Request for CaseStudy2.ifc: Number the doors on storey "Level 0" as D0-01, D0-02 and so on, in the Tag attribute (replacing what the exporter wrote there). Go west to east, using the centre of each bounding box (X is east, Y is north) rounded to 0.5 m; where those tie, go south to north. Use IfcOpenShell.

First a look at what the model holds.

```python
import ifcopenshell
import ifcopenshell.util.element
import ifcopenshell.util.placement

model = ifcopenshell.open("CaseStudy2.ifc")
print(model.schema)
storey = next(s for s in model.by_type("IfcBuildingStorey") if s.Name == "Level 0")
doors = [e for e in ifcopenshell.util.element.get_decomposition(storey) if e.is_a("IfcDoor")]
for e in sorted(doors, key=lambda e: e.id()):
    origin = ifcopenshell.util.placement.get_local_placement(e.ObjectPlacement)[:3, 3]
    print(e.id(), e.Tag, e.Name, origin.round(2) + 0.0, sep=" | ")
```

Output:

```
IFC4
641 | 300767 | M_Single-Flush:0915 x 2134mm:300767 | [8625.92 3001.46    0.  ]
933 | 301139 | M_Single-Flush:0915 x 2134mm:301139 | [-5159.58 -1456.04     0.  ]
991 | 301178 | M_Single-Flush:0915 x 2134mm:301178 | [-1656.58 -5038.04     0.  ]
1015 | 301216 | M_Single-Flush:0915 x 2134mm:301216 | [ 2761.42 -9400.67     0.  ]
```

```python
import ifcopenshell
import ifcopenshell.geom
import ifcopenshell.util.element
import ifcopenshell.util.shape

model = ifcopenshell.open("CaseStudy2.ifc")
settings = ifcopenshell.geom.settings()
settings.set("use-world-coords", True)


def centre(element):
    shape = ifcopenshell.geom.create_shape(settings, element)
    return ifcopenshell.util.shape.get_bbox_centroid(shape.geometry)


storey = next(s for s in model.by_type("IfcBuildingStorey") if s.Name == "Level 0")
doors = [e for e in ifcopenshell.util.element.get_decomposition(storey) if e.is_a("IfcDoor")]

# Insertion points can sit at a corner or the storey origin, so sort by the geometry (in metres).
centres = {e: centre(e) for e in doors}
doors.sort(key=lambda e: (round(centres[e][0] / 0.5), centres[e][1]))

for i, e in enumerate(doors, start=1):
    number = f"D0-{i:02d}"
    e.Tag = number
    print(e.id(), number)

model.write("CaseStudy2-out.ifc")
```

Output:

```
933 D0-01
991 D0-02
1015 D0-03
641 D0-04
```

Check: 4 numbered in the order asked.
